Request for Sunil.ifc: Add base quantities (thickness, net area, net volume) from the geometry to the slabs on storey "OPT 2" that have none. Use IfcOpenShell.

First a look at what the model holds.

```python
import ifcopenshell
import ifcopenshell.util.element
import ifcopenshell.util.unit

model = ifcopenshell.open("Sunil.ifc")
print(model.schema)
for unit_type in ("LENGTHUNIT", "AREAUNIT", "VOLUMEUNIT"):
    print(unit_type, ifcopenshell.util.unit.calculate_unit_scale(model, unit_type))
storey = next(s for s in model.by_type("IfcBuildingStorey") if s.Name == "OPT 2")
slabs = [e for e in ifcopenshell.util.element.get_decomposition(storey) if e.is_a("IfcSlab")]
for e in sorted(slabs, key=lambda e: e.id()):
    print(e.id(), e.is_a(), e.Name, list(ifcopenshell.util.element.get_psets(e, qtos_only=True)), sep=" | ")
```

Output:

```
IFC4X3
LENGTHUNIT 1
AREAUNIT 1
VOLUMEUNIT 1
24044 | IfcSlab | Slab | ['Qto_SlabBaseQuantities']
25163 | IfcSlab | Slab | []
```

```python
import ifcopenshell
import ifcopenshell.api.pset
import ifcopenshell.geom
import ifcopenshell.util.element
import ifcopenshell.util.shape
import ifcopenshell.util.unit

model = ifcopenshell.open("Sunil.ifc")
unit_scale = ifcopenshell.util.unit.calculate_unit_scale(model)
area_scale = ifcopenshell.util.unit.calculate_unit_scale(model, "AREAUNIT")
volume_scale = ifcopenshell.util.unit.calculate_unit_scale(model, "VOLUMEUNIT")
settings = ifcopenshell.geom.settings()

storey = next(s for s in model.by_type("IfcBuildingStorey") if s.Name == "OPT 2")
slabs = [e for e in ifcopenshell.util.element.get_decomposition(storey) if e.is_a("IfcSlab")]

for e in sorted(slabs, key=lambda e: e.id()):
    if ifcopenshell.util.element.get_psets(e, qtos_only=True, should_inherit=False):
        continue
    # Geometry comes back in metres, in the element's own axes.
    shape = ifcopenshell.geom.create_shape(settings, e)
    values = {
        "Width": ifcopenshell.util.shape.get_z(shape.geometry) / unit_scale,
        "NetArea": ifcopenshell.util.shape.get_footprint_area(shape.geometry) / area_scale,
        "NetVolume": ifcopenshell.util.shape.get_volume(shape.geometry) / volume_scale,
    }
    qto = ifcopenshell.api.pset.add_qto(model, product=e, name="Qto_SlabBaseQuantities")
    ifcopenshell.api.pset.edit_qto(model, qto=qto, properties=values)
    print(e.id(), {k: round(v, 3) for k, v in values.items()})

model.write("Sunil_updated.ifc")
```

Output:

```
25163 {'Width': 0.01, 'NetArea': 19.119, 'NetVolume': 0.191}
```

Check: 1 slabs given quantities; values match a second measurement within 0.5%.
